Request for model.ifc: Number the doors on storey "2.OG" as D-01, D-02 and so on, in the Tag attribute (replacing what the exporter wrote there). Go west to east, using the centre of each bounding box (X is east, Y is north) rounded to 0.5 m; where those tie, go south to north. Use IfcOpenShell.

First a look at what the model holds.

```python
import ifcopenshell
import ifcopenshell.util.element
import ifcopenshell.util.placement

model = ifcopenshell.open("model.ifc")
print(model.schema)
storey = next(s for s in model.by_type("IfcBuildingStorey") if s.Name == "2.OG")
doors = [e for e in ifcopenshell.util.element.get_decomposition(storey) if e.is_a("IfcDoor")]
for e in sorted(doors, key=lambda e: e.id()):
    origin = ifcopenshell.util.placement.get_local_placement(e.ObjectPlacement)[:3, 3]
    print(e.id(), e.Tag, e.Name, origin.round(2) + 0.0, sep=" | ")
```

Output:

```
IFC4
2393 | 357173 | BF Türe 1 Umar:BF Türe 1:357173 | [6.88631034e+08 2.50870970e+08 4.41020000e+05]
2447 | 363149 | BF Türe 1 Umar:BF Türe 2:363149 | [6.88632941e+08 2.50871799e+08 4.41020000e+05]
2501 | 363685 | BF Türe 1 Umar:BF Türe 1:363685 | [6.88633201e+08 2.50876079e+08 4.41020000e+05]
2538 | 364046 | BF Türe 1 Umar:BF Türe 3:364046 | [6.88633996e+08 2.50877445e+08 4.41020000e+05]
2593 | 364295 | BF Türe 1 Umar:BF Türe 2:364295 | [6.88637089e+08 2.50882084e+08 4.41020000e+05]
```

```python
import ifcopenshell
import ifcopenshell.geom
import ifcopenshell.util.element
import ifcopenshell.util.shape

model = ifcopenshell.open("model.ifc")
settings = ifcopenshell.geom.settings()
settings.set("use-world-coords", True)


def centre(element):
    shape = ifcopenshell.geom.create_shape(settings, element)
    return ifcopenshell.util.shape.get_bbox_centroid(shape.geometry)


storey = next(s for s in model.by_type("IfcBuildingStorey") if s.Name == "2.OG")
doors = [e for e in ifcopenshell.util.element.get_decomposition(storey) if e.is_a("IfcDoor")]

# Insertion points can sit at a corner or the storey origin, so sort by the geometry (in metres).
centres = {e: centre(e) for e in doors}
doors.sort(key=lambda e: (round(centres[e][0] / 0.5), centres[e][1]))

for i, e in enumerate(doors, start=1):
    number = f"D-{i:02d}"
    e.Tag = number
    print(e.id(), number)

model.write("model_updated.ifc")
```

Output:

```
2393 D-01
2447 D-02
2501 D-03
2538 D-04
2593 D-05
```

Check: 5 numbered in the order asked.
